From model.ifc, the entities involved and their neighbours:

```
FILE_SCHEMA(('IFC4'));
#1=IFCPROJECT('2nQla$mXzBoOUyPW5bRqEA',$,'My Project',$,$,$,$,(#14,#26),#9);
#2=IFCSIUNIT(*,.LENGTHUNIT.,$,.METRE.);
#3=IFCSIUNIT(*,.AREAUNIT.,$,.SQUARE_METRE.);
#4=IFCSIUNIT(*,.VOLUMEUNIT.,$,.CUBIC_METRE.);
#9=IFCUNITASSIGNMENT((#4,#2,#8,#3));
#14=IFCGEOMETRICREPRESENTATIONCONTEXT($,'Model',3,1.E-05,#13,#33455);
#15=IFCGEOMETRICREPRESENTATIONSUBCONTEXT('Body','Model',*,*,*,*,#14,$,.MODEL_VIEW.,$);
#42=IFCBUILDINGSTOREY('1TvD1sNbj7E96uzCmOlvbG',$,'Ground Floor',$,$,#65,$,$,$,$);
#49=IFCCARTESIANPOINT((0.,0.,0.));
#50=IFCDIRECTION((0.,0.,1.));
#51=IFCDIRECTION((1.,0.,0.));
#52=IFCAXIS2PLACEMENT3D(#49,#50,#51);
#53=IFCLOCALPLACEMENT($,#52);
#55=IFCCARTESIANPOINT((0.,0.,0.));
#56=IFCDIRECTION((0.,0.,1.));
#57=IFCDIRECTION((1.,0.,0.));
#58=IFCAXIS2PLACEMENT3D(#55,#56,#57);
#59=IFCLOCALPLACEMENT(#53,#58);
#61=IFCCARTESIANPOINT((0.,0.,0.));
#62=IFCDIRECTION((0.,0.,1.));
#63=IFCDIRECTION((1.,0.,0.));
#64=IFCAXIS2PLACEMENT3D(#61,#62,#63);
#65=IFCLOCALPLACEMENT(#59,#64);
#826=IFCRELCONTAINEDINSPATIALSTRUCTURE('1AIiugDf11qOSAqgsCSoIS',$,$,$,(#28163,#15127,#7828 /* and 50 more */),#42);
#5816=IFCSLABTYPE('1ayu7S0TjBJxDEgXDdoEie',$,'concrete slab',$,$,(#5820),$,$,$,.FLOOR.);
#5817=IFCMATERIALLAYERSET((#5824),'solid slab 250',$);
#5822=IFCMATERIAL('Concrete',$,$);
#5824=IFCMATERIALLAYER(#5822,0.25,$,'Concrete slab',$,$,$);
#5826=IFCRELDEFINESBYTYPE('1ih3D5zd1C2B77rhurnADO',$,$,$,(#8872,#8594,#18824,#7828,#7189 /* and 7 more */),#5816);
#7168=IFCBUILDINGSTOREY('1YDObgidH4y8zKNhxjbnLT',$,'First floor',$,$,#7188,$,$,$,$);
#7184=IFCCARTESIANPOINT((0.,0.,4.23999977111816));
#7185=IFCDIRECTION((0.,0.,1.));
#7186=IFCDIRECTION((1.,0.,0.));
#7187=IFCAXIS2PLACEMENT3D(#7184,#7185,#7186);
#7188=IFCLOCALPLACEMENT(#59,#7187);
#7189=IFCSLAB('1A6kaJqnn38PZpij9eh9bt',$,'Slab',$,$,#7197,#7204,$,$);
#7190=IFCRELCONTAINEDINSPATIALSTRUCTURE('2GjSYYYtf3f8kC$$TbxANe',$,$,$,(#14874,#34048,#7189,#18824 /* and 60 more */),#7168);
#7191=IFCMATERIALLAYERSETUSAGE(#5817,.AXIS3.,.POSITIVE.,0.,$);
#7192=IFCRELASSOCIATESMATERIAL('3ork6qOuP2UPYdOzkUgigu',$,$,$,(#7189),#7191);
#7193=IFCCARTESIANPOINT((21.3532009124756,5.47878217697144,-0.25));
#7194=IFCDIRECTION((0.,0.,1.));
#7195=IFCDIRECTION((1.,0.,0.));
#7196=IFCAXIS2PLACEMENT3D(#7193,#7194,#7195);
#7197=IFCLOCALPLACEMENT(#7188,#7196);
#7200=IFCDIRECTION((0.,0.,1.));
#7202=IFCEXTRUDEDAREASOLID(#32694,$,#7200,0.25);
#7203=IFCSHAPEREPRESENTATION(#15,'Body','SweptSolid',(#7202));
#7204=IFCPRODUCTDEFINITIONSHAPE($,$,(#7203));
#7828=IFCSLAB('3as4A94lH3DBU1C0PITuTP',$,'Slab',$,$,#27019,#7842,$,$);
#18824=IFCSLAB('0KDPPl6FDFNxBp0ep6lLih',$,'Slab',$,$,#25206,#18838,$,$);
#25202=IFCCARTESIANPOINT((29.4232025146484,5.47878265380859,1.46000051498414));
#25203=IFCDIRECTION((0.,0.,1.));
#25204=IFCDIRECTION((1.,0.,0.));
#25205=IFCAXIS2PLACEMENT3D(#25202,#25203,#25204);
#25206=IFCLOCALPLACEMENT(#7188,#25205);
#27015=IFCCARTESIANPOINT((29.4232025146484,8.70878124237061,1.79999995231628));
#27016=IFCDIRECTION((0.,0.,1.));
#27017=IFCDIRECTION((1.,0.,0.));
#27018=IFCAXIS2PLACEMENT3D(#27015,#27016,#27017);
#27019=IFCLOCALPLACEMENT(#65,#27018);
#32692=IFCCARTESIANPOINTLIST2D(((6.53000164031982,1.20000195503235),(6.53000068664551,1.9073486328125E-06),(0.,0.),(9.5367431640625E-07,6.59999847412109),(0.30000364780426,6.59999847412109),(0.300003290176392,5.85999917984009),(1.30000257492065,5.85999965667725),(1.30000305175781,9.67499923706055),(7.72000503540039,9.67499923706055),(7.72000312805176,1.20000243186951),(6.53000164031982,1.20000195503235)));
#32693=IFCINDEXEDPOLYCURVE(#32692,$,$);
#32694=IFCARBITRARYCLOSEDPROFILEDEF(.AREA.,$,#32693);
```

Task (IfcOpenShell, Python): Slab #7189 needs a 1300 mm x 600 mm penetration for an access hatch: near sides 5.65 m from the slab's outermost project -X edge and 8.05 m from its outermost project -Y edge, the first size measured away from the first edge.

```python
import numpy as np
import ifcopenshell
import ifcopenshell.api.feature
import ifcopenshell.api.geometry
import ifcopenshell.api.root
import ifcopenshell.geom
import ifcopenshell.util.placement
import ifcopenshell.util.representation
import ifcopenshell.util.shape
import ifcopenshell.util.unit

model = ifcopenshell.open("model.ifc")
unit_scale = ifcopenshell.util.unit.calculate_unit_scale(model)
settings = ifcopenshell.geom.settings()


def volume(element):
    """Net volume in cubic metres, openings subtracted."""
    shape = ifcopenshell.geom.create_shape(settings, element)
    return ifcopenshell.util.shape.get_volume(shape.geometry)


slab = model.by_guid("1A6kaJqnn38PZpij9eh9bt")
before = volume(slab)

# Extent in the slab's own axes, in metres. The edges named are its -X and -Y sides.
slab_shape = ifcopenshell.geom.create_shape(settings, slab)
vertices = ifcopenshell.util.shape.get_vertices(slab_shape.geometry)
x_min, y_min, bottom = vertices.min(axis=0)
top = vertices[:, 2].max()

opening = ifcopenshell.api.root.create_entity(model, ifc_class="IfcOpeningElement", name="Access hatch opening", predefined_type="OPENING")
context = ifcopenshell.util.representation.get_context(model, "Model", "Body", "MODEL_VIEW")
width, depth = 1.3, 0.6
outline = [(0.0, 0.0), (width, 0.0), (width, depth), (0.0, depth), (0.0, 0.0)]
# Overshoot both faces by 50 mm so the cut is clean.
shape = ifcopenshell.api.geometry.add_slab_representation(
    model, context=context, depth=top - bottom + 0.1, polyline=outline
)
ifcopenshell.api.geometry.assign_representation(model, product=opening, representation=shape)

matrix = ifcopenshell.util.placement.get_local_placement(slab.ObjectPlacement)
matrix[:, 3] = matrix @ np.append(np.array([x_min + 5.65, y_min + 8.05, bottom - 0.05]) / unit_scale, 1.0)
ifcopenshell.api.geometry.edit_object_placement(model, product=opening, matrix=matrix, is_si=False)
ifcopenshell.api.feature.add_feature(model, feature=opening, element=slab)

after = volume(slab)

print(f"slab volume {before:.3f} -> {after:.3f} m3")

model.write("model_v2.ifc")
```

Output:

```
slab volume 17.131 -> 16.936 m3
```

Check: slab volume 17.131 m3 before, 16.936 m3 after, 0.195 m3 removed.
